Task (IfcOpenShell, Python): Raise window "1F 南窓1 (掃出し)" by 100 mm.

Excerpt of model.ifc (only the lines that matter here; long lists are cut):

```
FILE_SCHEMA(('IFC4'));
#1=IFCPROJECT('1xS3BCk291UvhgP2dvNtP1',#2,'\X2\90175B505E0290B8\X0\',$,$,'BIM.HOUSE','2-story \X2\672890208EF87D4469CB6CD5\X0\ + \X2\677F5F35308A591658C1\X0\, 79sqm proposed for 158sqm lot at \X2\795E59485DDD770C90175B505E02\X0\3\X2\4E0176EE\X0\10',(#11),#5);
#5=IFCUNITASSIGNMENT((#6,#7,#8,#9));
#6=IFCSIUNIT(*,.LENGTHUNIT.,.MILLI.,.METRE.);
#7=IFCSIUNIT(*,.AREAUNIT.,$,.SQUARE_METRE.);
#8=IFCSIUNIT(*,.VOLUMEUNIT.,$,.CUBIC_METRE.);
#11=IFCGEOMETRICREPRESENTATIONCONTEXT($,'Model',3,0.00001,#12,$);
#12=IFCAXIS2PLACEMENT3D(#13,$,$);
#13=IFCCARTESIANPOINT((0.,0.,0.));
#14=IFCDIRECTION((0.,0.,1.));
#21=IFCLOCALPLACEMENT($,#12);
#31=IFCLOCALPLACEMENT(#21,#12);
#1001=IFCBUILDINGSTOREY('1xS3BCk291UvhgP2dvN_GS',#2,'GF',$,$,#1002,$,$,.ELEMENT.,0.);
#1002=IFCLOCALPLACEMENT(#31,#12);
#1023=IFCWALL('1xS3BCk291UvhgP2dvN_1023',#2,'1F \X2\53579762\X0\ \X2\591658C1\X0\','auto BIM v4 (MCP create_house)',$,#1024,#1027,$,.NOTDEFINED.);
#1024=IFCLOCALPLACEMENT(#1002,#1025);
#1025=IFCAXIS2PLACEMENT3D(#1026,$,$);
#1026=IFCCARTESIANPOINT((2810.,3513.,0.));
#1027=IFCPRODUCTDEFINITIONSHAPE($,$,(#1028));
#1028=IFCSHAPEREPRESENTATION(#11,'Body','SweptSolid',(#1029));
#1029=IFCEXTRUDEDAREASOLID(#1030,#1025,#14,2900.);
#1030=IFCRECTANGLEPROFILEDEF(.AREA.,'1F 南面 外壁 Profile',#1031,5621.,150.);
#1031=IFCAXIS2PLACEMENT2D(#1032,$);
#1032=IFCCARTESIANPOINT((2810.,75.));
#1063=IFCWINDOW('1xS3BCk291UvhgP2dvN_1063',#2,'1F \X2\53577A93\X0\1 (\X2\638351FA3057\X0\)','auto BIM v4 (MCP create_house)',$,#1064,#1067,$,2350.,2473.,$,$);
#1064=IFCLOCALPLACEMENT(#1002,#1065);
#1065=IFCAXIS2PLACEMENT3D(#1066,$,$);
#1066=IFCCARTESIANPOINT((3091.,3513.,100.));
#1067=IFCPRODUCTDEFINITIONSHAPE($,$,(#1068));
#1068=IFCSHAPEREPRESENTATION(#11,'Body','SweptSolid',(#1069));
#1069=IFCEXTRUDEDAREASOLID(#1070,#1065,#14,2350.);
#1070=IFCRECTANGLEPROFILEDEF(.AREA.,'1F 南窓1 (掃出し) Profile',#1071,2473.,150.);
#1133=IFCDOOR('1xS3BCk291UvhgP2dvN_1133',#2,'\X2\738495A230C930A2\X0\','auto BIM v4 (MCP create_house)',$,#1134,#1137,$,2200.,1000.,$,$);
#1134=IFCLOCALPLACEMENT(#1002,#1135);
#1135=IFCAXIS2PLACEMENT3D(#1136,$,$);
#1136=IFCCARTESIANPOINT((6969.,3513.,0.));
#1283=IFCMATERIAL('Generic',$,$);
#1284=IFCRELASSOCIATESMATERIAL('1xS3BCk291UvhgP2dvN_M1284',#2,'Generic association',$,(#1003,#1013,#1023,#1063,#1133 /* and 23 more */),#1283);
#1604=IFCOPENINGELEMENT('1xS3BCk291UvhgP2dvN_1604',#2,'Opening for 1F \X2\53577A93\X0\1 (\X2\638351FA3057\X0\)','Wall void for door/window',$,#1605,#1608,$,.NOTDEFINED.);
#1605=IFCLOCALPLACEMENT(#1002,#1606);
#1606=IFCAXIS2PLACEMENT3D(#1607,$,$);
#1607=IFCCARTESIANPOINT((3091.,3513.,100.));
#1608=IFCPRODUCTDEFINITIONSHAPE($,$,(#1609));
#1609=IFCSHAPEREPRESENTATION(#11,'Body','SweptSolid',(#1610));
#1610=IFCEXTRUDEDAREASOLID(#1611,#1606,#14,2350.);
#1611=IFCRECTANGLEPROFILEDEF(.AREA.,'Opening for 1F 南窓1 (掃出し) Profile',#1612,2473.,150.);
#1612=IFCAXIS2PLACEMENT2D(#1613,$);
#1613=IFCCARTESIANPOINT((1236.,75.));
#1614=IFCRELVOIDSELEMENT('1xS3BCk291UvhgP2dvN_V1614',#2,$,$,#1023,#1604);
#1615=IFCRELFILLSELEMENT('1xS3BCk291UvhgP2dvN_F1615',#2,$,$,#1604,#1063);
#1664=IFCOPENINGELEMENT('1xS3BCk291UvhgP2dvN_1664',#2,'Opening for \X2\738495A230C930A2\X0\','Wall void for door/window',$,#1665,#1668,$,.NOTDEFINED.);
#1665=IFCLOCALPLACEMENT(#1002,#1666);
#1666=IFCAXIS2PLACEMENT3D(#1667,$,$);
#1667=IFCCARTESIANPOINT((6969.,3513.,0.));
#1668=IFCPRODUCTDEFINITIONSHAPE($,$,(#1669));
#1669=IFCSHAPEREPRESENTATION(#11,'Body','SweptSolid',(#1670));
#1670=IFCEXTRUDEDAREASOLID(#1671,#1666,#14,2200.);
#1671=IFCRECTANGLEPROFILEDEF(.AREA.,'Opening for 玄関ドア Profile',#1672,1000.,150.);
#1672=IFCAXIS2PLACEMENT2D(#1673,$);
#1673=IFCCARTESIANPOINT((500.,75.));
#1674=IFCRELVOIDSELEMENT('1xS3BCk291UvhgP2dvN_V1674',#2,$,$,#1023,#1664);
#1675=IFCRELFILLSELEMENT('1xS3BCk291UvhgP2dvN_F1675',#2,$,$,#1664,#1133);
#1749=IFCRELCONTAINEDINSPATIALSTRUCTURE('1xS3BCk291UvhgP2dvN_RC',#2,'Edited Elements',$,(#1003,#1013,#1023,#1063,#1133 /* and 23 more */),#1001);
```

```python
import numpy as np
import ifcopenshell
import ifcopenshell.api.geometry
import ifcopenshell.util.placement
import ifcopenshell.util.unit

model = ifcopenshell.open("model.ifc")
unit_scale = ifcopenshell.util.unit.calculate_unit_scale(model)

window = model.by_guid("1xS3BCk291UvhgP2dvN_1063")
opening = window.FillsVoids[0].RelatingOpeningElement
dz = 100.0

shift = np.array([0.0, 0.0, dz])
# The window is not placed relative to its opening, so move both.
for product in (opening, window):
    matrix = ifcopenshell.util.placement.get_local_placement(product.ObjectPlacement)
    matrix[:3, 3] += shift
    ifcopenshell.api.geometry.edit_object_placement(model, product=product, matrix=matrix, is_si=False)

print(f"moved by {dz * unit_scale:+.3f} m")

model.write("model_rev.ifc")
```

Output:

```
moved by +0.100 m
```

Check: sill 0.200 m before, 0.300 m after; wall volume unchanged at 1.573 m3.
